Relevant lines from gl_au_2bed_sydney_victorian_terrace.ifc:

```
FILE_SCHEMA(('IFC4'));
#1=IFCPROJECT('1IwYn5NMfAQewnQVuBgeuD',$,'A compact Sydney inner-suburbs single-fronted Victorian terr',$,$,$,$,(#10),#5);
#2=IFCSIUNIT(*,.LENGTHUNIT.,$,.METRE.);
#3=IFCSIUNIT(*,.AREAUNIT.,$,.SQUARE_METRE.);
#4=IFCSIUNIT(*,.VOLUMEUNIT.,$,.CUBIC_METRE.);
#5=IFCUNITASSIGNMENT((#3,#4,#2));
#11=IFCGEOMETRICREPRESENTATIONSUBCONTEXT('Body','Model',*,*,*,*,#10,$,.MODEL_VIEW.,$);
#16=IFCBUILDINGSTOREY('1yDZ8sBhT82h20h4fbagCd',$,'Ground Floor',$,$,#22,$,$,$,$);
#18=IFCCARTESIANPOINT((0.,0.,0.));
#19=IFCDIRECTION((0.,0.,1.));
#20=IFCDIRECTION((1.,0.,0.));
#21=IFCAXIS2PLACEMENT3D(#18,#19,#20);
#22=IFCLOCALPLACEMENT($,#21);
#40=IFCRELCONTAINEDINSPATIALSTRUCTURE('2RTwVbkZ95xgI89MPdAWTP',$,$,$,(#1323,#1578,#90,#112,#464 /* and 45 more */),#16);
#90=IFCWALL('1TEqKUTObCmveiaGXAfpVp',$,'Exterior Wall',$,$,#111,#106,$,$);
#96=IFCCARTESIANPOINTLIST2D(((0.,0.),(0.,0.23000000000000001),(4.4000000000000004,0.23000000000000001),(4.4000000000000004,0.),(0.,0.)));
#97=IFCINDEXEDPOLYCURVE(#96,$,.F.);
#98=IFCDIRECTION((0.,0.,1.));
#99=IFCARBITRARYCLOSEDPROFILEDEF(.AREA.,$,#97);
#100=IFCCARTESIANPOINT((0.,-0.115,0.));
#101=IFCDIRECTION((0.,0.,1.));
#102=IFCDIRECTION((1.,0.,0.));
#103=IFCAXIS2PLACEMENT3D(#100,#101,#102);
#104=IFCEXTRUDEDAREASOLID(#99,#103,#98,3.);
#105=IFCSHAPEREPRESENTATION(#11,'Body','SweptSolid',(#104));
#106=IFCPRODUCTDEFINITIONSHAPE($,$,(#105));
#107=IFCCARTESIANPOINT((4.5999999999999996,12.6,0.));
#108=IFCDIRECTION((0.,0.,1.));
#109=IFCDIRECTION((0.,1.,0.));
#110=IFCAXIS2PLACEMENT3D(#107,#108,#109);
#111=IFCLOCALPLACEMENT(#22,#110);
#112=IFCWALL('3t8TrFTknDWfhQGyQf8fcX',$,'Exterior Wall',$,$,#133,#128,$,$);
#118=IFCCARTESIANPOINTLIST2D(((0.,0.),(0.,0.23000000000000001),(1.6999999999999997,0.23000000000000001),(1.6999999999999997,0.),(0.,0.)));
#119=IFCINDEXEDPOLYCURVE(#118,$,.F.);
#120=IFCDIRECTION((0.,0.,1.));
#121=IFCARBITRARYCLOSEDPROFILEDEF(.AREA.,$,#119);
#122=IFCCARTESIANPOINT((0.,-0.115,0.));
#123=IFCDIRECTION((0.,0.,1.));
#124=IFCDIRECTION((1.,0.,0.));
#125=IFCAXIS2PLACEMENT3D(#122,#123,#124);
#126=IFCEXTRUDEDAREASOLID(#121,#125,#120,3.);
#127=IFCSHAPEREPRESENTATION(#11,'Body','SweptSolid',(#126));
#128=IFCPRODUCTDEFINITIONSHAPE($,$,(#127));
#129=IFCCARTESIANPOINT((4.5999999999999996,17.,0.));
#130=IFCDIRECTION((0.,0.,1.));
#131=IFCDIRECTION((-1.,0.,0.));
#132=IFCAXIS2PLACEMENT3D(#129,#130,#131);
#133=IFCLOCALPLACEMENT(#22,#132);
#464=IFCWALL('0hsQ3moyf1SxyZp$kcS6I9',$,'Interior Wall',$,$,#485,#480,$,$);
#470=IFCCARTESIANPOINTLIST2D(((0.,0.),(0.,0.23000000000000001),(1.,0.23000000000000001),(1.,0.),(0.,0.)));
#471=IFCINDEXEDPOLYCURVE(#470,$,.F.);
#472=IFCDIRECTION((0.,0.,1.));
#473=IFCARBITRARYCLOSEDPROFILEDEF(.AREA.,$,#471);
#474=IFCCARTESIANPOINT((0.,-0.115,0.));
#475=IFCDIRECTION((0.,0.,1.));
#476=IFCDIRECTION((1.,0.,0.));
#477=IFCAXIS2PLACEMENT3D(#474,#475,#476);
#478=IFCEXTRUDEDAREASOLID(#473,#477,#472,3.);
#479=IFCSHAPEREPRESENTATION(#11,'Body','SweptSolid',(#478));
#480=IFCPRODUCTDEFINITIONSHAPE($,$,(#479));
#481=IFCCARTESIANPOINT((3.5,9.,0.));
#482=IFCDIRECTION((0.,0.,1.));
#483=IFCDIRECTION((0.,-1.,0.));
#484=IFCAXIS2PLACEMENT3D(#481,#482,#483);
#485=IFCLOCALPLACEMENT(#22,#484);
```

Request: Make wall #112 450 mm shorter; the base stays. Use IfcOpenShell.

```python
import ifcopenshell
import ifcopenshell.geom
import ifcopenshell.util.representation
import ifcopenshell.util.shape
import ifcopenshell.util.unit

model = ifcopenshell.open("gl_au_2bed_sydney_victorian_terrace.ifc")
unit_scale = ifcopenshell.util.unit.calculate_unit_scale(model)
settings = ifcopenshell.geom.settings()


def volume(element):
    """Net volume in cubic metres, openings subtracted."""
    shape = ifcopenshell.geom.create_shape(settings, element)
    return ifcopenshell.util.shape.get_volume(shape.geometry)


wall = model.by_id(112)
before = volume(wall)

body = ifcopenshell.util.representation.get_representation(wall, "Model", "Body")
solid = body.Items[0]
old_height = solid.Depth
solid.Depth -= 0.45 / unit_scale
after = volume(wall)

print(f"height {old_height:g} -> {solid.Depth:g}, volume {before:.3f} -> {after:.3f} m3")

model.write("gl_au_2bed_sydney_victorian_terrace_rev.ifc")
```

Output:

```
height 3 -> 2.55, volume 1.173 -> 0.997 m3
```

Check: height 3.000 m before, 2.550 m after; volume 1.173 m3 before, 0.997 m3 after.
